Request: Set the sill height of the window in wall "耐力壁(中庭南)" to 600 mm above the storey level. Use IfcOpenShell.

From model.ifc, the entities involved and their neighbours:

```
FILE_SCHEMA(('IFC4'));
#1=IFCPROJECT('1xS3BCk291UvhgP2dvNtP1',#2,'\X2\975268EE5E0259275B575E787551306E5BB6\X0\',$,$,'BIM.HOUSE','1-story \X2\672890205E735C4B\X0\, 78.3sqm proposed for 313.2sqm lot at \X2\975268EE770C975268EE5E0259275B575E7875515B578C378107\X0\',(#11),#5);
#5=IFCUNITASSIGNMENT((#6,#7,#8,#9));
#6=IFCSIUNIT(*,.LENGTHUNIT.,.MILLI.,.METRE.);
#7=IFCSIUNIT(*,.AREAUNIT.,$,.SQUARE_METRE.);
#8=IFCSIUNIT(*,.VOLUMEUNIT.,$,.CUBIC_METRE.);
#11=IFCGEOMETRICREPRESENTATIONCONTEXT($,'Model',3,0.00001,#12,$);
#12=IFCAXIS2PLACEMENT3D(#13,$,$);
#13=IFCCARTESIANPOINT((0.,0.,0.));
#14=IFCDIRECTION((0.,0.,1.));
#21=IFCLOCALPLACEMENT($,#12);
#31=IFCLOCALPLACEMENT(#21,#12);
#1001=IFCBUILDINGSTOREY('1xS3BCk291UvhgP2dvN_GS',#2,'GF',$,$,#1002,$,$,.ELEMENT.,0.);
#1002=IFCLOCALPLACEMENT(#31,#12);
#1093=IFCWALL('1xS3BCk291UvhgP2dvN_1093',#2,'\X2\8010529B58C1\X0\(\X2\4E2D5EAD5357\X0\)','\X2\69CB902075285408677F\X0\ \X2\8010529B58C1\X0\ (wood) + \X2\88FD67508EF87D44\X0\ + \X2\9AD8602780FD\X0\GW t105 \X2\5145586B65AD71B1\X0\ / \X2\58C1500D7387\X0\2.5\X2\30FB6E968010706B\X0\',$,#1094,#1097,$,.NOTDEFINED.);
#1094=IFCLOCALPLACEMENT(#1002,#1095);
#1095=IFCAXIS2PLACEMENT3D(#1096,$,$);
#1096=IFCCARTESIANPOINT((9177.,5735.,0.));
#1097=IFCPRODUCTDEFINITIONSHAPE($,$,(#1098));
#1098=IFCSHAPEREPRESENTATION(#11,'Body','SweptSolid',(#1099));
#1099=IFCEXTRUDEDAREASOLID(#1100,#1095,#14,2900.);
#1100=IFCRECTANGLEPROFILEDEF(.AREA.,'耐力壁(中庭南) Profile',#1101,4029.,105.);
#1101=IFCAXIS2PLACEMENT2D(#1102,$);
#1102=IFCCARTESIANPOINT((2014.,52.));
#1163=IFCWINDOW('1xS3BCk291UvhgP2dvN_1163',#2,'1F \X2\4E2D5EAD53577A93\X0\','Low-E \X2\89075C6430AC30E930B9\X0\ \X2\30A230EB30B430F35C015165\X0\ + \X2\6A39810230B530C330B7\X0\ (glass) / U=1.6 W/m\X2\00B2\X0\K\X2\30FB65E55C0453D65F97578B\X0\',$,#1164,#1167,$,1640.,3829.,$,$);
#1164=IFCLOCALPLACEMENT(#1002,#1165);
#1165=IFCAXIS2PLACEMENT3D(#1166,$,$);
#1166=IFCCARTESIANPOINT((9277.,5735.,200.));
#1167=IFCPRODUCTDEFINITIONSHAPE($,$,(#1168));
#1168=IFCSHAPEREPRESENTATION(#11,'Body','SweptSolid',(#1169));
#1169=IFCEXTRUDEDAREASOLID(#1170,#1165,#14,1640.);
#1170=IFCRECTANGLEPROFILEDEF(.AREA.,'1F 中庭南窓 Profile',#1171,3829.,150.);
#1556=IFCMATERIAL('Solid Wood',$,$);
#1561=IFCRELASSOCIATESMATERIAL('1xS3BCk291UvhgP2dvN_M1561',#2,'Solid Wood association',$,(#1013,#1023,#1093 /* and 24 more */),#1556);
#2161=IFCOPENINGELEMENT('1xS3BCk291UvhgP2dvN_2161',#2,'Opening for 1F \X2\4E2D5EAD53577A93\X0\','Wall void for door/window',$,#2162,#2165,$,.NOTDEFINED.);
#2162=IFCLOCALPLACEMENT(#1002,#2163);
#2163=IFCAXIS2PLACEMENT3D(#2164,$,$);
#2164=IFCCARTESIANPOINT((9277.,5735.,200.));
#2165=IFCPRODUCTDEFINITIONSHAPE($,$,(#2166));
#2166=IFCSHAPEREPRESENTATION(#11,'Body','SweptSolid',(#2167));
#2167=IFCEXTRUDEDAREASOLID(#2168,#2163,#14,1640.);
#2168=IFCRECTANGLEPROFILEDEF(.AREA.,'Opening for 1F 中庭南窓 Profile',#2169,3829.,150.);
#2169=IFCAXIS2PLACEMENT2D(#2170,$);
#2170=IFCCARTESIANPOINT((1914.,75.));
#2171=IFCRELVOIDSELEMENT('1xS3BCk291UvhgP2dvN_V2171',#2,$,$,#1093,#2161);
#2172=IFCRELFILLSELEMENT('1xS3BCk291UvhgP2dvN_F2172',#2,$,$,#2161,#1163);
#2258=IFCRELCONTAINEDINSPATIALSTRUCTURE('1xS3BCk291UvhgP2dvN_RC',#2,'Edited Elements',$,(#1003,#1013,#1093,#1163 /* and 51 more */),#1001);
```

```python
import numpy as np
import ifcopenshell
import ifcopenshell.api.geometry
import ifcopenshell.geom
import ifcopenshell.util.element
import ifcopenshell.util.placement
import ifcopenshell.util.shape
import ifcopenshell.util.unit

model = ifcopenshell.open("model.ifc")
unit_scale = ifcopenshell.util.unit.calculate_unit_scale(model)

window = model.by_guid("1xS3BCk291UvhgP2dvN_1163")
opening = window.FillsVoids[0].RelatingOpeningElement
storey = ifcopenshell.util.element.get_container(window, ifc_class="IfcBuildingStorey")
level = ifcopenshell.util.placement.get_local_placement(storey.ObjectPlacement)[2, 3]

# The opening's origin need not be at the sill, so measure its lowest point.
shape = ifcopenshell.geom.create_shape(ifcopenshell.geom.settings(), opening)
bottom = ifcopenshell.util.shape.get_shape_bottom_elevation(shape, shape.geometry) / unit_scale
dz = level + 600.0 - bottom

shift = np.array([0.0, 0.0, dz])
# The window is not placed relative to its opening, so move both.
for product in (opening, window):
    matrix = ifcopenshell.util.placement.get_local_placement(product.ObjectPlacement)
    matrix[:3, 3] += shift
    ifcopenshell.api.geometry.edit_object_placement(model, product=product, matrix=matrix, is_si=False)

print(f"moved by {dz * unit_scale:+.3f} m")

model.write("model-out.ifc")
```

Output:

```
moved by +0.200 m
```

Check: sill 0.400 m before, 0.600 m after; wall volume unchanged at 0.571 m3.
